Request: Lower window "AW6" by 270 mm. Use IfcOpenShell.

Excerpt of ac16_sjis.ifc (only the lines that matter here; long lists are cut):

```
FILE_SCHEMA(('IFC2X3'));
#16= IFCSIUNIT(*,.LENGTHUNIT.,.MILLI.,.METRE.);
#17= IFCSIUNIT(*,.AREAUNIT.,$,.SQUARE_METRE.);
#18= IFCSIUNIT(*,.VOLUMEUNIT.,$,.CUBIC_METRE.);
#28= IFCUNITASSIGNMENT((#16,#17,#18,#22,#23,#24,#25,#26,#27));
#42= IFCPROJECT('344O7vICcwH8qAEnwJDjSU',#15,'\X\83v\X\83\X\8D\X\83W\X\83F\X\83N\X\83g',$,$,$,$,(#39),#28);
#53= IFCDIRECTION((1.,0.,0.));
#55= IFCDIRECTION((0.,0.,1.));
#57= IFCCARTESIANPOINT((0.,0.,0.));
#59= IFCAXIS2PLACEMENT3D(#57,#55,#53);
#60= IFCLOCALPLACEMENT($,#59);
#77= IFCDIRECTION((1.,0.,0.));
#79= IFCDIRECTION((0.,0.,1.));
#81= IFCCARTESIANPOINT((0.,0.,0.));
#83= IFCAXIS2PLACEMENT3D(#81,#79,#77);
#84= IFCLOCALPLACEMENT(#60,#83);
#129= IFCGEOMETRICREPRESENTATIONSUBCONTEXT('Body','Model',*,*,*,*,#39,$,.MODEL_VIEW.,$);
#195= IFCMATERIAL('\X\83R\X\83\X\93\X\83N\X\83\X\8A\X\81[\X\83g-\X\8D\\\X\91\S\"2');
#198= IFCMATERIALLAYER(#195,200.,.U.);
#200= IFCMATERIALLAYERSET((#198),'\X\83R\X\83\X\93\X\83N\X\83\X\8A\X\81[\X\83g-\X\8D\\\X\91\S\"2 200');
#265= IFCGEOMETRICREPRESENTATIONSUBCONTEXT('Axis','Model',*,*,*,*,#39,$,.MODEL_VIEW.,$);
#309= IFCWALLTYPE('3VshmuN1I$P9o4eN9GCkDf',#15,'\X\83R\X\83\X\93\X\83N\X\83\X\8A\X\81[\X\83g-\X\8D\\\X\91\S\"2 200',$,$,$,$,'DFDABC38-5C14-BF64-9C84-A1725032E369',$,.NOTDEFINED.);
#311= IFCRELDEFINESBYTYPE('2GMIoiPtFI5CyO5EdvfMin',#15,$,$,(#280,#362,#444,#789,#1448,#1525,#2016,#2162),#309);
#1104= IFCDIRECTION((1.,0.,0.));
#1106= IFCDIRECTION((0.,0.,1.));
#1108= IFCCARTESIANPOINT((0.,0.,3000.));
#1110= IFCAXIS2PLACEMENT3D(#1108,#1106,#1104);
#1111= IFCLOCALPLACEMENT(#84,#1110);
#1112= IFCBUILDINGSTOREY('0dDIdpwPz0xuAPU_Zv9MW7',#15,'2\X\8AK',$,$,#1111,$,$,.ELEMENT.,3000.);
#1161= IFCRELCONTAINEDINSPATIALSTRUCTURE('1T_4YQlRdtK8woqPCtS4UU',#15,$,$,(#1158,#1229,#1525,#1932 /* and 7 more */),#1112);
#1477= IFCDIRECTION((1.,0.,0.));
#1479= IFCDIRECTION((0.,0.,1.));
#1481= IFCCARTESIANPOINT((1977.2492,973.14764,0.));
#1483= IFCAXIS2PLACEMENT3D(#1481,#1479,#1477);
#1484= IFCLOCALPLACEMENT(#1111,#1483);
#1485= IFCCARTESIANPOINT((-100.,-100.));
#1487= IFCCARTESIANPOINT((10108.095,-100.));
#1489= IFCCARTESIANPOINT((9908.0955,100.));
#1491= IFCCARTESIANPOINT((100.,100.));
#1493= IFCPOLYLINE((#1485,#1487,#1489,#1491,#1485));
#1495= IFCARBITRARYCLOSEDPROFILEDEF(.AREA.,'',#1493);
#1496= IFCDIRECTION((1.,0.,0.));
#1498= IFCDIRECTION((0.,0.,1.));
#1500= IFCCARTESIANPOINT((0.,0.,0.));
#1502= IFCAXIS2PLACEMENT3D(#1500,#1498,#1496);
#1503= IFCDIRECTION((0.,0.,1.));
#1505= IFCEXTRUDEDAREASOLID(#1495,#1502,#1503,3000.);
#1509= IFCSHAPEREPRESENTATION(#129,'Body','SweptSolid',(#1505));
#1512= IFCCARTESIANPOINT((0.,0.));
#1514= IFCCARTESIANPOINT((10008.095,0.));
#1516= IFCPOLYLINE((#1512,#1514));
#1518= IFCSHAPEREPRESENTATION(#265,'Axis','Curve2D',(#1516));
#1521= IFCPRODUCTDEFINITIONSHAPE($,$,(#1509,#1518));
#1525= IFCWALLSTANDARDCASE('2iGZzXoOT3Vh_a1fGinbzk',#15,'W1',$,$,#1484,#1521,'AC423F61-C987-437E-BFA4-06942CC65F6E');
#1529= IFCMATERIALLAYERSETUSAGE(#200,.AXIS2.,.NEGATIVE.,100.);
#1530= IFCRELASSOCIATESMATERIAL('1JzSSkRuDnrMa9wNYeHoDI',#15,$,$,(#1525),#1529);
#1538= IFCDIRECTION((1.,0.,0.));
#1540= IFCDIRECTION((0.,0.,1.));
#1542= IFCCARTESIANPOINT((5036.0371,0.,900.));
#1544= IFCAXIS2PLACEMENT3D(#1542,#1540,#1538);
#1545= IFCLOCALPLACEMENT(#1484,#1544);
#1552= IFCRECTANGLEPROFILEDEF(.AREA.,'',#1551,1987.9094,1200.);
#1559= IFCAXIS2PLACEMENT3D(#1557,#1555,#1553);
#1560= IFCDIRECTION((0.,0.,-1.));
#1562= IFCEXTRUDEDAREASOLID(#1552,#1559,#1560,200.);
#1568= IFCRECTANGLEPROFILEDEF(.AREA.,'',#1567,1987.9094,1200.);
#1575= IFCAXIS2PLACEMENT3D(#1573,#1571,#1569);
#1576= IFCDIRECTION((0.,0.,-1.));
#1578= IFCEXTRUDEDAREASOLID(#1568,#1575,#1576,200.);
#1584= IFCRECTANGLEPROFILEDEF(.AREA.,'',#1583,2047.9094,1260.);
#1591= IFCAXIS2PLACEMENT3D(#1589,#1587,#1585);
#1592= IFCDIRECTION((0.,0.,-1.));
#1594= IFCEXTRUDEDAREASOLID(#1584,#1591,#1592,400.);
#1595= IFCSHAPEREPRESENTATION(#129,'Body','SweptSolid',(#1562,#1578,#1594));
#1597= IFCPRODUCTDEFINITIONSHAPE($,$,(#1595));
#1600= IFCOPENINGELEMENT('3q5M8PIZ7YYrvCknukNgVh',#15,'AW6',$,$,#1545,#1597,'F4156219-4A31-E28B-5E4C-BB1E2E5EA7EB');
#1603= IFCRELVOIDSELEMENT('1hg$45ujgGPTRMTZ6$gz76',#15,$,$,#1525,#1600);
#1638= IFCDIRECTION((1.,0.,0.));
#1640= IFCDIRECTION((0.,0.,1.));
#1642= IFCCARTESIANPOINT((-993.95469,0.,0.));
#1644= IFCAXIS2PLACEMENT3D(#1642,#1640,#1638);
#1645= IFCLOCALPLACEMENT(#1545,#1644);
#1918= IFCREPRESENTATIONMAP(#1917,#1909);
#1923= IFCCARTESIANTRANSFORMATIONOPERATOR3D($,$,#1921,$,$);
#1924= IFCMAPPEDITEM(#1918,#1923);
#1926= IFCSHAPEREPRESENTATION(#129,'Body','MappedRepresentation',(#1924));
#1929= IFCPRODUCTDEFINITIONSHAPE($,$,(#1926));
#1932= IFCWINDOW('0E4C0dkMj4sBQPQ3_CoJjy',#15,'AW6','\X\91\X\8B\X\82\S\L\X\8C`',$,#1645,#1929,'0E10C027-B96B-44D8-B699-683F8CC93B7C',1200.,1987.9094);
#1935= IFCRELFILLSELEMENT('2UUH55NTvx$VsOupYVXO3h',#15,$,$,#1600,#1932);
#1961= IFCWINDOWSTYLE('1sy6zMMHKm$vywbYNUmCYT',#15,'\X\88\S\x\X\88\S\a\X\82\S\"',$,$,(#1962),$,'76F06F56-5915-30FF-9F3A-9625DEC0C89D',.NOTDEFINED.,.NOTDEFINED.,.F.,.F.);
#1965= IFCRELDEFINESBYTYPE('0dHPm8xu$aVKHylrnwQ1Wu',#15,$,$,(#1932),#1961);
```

```python
import numpy as np
import ifcopenshell
import ifcopenshell.api.geometry
import ifcopenshell.util.placement
import ifcopenshell.util.unit

model = ifcopenshell.open("ac16_sjis.ifc")
unit_scale = ifcopenshell.util.unit.calculate_unit_scale(model)

window = model.by_guid("0E4C0dkMj4sBQPQ3_CoJjy")
opening = window.FillsVoids[0].RelatingOpeningElement
dz = -270.0

shift = np.array([0.0, 0.0, dz])
# The window is placed relative to its opening, so it follows when the opening moves.
matrix = ifcopenshell.util.placement.get_local_placement(opening.ObjectPlacement)
matrix[:3, 3] += shift
ifcopenshell.api.geometry.edit_object_placement(
    model, product=opening, matrix=matrix, is_si=False, should_transform_children=True
)

print(f"moved by {dz * unit_scale:+.3f} m")

model.write("ac16_sjis_updated.ifc")
```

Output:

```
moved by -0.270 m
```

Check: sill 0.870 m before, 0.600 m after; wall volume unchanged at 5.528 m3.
